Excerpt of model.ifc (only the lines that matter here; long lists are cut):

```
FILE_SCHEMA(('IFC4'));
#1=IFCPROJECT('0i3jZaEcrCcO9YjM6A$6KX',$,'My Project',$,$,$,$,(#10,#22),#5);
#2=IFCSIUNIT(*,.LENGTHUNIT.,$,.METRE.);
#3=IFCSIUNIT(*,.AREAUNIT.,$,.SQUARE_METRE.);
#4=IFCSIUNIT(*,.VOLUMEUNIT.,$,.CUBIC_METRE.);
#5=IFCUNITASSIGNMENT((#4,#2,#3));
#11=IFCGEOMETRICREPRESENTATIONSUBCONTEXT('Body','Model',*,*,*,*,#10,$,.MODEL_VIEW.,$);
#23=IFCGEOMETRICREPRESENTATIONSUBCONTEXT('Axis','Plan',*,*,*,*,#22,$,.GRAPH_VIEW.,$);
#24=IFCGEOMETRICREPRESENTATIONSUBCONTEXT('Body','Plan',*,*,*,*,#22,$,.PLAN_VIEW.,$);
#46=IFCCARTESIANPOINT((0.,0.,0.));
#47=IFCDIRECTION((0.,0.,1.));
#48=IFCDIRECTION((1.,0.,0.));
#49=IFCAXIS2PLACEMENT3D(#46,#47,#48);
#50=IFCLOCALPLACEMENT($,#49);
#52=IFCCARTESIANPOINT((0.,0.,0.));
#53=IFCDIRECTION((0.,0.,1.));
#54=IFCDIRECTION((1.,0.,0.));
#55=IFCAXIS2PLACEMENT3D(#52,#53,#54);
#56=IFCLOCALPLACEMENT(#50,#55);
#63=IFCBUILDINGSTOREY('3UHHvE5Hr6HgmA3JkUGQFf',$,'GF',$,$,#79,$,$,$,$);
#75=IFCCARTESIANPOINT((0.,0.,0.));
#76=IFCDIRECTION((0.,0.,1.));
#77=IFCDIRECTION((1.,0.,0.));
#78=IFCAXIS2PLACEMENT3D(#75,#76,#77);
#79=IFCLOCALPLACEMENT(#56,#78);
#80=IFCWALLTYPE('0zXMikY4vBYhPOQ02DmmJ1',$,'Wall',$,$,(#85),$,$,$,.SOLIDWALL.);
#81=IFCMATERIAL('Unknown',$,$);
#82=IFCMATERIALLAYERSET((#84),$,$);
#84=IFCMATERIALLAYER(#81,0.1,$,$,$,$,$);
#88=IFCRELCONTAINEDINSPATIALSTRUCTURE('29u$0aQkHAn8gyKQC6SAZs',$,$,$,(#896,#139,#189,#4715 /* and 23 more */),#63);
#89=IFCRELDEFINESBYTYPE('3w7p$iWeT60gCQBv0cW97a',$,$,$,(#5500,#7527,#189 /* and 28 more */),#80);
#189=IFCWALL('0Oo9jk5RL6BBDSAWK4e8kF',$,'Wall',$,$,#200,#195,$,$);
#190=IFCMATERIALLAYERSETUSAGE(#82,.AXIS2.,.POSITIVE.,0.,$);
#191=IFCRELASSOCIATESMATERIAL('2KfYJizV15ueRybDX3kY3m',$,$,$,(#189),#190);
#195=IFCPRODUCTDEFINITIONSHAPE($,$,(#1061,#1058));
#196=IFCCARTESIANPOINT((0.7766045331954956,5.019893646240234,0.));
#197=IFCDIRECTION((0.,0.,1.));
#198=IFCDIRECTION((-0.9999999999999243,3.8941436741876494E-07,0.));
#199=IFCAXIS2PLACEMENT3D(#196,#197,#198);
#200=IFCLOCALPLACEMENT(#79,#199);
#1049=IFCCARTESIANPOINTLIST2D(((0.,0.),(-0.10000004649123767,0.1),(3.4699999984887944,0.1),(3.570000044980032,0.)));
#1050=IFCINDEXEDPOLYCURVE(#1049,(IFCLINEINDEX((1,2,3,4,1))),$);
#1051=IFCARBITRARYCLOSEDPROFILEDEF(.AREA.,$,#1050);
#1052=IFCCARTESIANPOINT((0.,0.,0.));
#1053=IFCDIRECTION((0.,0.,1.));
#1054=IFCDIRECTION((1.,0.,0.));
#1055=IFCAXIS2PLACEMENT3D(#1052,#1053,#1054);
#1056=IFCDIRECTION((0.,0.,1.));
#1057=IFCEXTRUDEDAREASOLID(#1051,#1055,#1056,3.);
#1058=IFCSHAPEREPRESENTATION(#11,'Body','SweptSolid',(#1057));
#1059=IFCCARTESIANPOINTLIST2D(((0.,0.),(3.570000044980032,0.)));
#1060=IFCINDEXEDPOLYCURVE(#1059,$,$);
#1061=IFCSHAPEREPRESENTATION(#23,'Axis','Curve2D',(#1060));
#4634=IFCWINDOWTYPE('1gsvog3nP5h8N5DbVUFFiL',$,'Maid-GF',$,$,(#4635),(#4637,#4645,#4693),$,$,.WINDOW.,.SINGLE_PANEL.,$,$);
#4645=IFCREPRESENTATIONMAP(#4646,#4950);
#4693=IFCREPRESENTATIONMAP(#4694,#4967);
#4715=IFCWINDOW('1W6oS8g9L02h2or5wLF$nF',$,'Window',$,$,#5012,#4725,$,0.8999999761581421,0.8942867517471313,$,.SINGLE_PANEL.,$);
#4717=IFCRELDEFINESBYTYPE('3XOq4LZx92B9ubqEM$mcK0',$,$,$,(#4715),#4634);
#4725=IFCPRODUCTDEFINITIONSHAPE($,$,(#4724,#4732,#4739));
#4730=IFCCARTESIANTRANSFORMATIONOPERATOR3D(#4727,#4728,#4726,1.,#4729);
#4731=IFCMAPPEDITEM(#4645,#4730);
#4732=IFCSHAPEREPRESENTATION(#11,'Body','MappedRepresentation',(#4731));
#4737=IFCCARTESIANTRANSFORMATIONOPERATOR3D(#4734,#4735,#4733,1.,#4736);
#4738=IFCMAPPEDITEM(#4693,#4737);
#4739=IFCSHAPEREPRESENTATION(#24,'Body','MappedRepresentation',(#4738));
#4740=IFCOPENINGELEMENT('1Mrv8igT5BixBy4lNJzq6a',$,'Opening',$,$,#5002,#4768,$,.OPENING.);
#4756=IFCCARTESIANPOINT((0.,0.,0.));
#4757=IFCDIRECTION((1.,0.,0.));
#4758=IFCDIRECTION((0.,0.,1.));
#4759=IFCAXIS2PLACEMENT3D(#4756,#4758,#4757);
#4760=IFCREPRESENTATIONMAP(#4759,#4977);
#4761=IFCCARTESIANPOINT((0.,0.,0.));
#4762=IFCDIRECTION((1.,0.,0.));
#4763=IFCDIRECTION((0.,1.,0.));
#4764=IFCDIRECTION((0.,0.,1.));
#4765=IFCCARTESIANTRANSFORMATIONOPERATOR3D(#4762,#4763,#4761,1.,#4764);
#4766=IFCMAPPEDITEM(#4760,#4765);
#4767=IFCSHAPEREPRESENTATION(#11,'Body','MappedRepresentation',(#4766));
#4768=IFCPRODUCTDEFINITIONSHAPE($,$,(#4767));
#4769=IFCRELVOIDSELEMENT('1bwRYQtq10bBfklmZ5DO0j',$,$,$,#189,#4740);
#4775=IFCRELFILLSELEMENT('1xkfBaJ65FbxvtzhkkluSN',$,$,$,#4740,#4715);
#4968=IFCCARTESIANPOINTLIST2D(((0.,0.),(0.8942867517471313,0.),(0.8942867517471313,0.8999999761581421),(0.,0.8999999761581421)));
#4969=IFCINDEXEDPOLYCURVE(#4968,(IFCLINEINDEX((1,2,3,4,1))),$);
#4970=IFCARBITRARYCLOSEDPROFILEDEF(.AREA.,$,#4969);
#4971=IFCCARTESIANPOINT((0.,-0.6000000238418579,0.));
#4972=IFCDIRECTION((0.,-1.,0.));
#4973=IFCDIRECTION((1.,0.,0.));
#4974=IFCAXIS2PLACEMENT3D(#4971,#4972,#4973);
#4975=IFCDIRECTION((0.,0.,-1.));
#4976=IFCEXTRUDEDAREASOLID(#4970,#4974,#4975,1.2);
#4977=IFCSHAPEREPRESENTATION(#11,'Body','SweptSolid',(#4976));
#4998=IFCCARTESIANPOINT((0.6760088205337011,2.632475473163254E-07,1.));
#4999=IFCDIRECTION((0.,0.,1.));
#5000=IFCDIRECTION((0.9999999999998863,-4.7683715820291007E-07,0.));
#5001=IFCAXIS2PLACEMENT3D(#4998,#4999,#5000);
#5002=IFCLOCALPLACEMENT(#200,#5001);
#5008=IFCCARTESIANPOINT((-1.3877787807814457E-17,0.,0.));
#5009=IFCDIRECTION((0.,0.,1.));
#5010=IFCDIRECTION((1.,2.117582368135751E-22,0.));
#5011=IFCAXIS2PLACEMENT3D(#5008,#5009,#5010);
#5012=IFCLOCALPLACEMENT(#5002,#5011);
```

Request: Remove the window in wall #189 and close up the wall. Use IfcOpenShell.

```python
import ifcopenshell
import ifcopenshell.api.feature
import ifcopenshell.api.root
import ifcopenshell.geom
import ifcopenshell.util.shape

model = ifcopenshell.open("model.ifc")
settings = ifcopenshell.geom.settings()


def volume(element):
    """Net volume in cubic metres, openings subtracted."""
    shape = ifcopenshell.geom.create_shape(settings, element)
    return ifcopenshell.util.shape.get_volume(shape.geometry)


window = model.by_guid("1W6oS8g9L02h2or5wLF$nF")
opening = window.FillsVoids[0].RelatingOpeningElement
wall = opening.VoidsElements[0].RelatingBuildingElement
before = volume(wall)

ifcopenshell.api.root.remove_product(model, product=window)
ifcopenshell.api.feature.remove_feature(model, feature=opening)

after = volume(wall)

print(f"wall volume {before:.3f} -> {after:.3f} m3")

model.write("model_edited.ifc")
```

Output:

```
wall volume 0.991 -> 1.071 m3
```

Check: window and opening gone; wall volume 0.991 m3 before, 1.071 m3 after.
